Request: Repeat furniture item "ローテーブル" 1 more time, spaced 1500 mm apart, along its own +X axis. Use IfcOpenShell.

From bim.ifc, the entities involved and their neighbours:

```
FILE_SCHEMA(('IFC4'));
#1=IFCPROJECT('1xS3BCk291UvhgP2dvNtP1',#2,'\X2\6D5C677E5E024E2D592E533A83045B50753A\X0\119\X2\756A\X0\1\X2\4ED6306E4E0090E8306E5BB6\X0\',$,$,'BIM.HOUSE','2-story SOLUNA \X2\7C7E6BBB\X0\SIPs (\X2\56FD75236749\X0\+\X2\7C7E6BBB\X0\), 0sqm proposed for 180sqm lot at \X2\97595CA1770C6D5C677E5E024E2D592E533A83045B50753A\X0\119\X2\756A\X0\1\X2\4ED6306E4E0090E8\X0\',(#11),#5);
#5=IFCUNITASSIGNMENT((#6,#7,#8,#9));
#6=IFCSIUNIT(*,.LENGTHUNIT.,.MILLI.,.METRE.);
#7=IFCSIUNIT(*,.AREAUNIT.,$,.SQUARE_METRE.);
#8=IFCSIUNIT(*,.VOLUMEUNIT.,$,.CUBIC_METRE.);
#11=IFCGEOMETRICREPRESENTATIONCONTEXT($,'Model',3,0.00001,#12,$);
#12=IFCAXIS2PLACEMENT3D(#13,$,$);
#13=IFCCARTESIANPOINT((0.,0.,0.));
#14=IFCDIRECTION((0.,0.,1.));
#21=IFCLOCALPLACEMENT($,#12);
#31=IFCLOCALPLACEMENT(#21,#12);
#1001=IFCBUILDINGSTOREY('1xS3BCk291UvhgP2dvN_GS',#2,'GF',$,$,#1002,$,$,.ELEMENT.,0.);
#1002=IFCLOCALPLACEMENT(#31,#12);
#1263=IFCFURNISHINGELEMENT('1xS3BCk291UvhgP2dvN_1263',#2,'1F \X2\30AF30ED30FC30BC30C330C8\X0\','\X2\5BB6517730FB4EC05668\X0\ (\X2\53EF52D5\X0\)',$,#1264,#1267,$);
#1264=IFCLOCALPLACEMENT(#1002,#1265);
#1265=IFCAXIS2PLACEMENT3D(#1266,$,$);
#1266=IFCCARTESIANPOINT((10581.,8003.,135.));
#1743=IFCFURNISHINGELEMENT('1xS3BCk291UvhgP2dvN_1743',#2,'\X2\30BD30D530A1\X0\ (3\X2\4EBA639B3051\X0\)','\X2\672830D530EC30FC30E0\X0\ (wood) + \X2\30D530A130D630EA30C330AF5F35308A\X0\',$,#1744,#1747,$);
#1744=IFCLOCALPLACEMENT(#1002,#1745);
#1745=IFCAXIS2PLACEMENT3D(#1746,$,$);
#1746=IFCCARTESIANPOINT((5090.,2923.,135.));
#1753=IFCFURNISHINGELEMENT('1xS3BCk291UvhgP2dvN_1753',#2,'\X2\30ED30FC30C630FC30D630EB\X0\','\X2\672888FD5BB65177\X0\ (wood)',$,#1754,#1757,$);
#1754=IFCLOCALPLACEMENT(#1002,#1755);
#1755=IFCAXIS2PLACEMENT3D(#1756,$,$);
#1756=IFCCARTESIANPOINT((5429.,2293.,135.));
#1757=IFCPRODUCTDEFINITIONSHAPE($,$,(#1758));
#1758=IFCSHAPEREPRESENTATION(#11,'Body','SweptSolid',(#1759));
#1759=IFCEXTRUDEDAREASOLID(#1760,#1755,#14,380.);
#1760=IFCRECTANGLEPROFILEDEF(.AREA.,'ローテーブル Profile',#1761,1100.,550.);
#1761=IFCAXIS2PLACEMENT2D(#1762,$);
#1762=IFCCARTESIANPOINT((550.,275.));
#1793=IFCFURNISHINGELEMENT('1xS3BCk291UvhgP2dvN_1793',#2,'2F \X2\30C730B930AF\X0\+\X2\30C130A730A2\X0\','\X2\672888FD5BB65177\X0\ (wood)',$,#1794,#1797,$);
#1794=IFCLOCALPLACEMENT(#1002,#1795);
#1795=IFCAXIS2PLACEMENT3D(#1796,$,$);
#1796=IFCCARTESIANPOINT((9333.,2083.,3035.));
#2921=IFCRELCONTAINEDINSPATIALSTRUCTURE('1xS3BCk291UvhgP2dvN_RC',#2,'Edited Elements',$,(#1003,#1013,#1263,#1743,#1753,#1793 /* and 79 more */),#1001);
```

```python
import ifcopenshell
import ifcopenshell.api.geometry
import ifcopenshell.api.root
import ifcopenshell.util.element
import ifcopenshell.util.placement

model = ifcopenshell.open("bim.ifc")


def reuse_history(source, copy):
    """copy_class also copies each property set's owner history, people and application; keep the originals."""
    for rel in copy.IsDefinedBy:
        if rel.is_a("IfcRelDefinesByProperties") and (history := rel.RelatingPropertyDefinition.OwnerHistory):
            rel.RelatingPropertyDefinition.OwnerHistory = source.OwnerHistory
            ifcopenshell.util.element.remove_deep2(model, history)


source = model.by_guid("1xS3BCk291UvhgP2dvN_1753")
base = ifcopenshell.util.placement.get_local_placement(source.ObjectPlacement)
step = base[:3, 0] * 1500.0

for i in range(1, 2):
    copy = ifcopenshell.api.root.copy_class(model, product=source)
    copy.Representation = ifcopenshell.util.element.copy_deep(
        model, source.Representation, exclude=["IfcGeometricRepresentationContext", "IfcRepresentationMap"]
    )
    reuse_history(source, copy)
    matrix = base.copy()
    matrix[:3, 3] += i * step
    print("added at", matrix[:3, 3].round(3) + 0.0)
    ifcopenshell.api.geometry.edit_object_placement(model, product=copy, matrix=matrix, is_si=False)

model.write("bim_updated.ifc")
```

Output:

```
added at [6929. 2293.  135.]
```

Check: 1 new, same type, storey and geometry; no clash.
